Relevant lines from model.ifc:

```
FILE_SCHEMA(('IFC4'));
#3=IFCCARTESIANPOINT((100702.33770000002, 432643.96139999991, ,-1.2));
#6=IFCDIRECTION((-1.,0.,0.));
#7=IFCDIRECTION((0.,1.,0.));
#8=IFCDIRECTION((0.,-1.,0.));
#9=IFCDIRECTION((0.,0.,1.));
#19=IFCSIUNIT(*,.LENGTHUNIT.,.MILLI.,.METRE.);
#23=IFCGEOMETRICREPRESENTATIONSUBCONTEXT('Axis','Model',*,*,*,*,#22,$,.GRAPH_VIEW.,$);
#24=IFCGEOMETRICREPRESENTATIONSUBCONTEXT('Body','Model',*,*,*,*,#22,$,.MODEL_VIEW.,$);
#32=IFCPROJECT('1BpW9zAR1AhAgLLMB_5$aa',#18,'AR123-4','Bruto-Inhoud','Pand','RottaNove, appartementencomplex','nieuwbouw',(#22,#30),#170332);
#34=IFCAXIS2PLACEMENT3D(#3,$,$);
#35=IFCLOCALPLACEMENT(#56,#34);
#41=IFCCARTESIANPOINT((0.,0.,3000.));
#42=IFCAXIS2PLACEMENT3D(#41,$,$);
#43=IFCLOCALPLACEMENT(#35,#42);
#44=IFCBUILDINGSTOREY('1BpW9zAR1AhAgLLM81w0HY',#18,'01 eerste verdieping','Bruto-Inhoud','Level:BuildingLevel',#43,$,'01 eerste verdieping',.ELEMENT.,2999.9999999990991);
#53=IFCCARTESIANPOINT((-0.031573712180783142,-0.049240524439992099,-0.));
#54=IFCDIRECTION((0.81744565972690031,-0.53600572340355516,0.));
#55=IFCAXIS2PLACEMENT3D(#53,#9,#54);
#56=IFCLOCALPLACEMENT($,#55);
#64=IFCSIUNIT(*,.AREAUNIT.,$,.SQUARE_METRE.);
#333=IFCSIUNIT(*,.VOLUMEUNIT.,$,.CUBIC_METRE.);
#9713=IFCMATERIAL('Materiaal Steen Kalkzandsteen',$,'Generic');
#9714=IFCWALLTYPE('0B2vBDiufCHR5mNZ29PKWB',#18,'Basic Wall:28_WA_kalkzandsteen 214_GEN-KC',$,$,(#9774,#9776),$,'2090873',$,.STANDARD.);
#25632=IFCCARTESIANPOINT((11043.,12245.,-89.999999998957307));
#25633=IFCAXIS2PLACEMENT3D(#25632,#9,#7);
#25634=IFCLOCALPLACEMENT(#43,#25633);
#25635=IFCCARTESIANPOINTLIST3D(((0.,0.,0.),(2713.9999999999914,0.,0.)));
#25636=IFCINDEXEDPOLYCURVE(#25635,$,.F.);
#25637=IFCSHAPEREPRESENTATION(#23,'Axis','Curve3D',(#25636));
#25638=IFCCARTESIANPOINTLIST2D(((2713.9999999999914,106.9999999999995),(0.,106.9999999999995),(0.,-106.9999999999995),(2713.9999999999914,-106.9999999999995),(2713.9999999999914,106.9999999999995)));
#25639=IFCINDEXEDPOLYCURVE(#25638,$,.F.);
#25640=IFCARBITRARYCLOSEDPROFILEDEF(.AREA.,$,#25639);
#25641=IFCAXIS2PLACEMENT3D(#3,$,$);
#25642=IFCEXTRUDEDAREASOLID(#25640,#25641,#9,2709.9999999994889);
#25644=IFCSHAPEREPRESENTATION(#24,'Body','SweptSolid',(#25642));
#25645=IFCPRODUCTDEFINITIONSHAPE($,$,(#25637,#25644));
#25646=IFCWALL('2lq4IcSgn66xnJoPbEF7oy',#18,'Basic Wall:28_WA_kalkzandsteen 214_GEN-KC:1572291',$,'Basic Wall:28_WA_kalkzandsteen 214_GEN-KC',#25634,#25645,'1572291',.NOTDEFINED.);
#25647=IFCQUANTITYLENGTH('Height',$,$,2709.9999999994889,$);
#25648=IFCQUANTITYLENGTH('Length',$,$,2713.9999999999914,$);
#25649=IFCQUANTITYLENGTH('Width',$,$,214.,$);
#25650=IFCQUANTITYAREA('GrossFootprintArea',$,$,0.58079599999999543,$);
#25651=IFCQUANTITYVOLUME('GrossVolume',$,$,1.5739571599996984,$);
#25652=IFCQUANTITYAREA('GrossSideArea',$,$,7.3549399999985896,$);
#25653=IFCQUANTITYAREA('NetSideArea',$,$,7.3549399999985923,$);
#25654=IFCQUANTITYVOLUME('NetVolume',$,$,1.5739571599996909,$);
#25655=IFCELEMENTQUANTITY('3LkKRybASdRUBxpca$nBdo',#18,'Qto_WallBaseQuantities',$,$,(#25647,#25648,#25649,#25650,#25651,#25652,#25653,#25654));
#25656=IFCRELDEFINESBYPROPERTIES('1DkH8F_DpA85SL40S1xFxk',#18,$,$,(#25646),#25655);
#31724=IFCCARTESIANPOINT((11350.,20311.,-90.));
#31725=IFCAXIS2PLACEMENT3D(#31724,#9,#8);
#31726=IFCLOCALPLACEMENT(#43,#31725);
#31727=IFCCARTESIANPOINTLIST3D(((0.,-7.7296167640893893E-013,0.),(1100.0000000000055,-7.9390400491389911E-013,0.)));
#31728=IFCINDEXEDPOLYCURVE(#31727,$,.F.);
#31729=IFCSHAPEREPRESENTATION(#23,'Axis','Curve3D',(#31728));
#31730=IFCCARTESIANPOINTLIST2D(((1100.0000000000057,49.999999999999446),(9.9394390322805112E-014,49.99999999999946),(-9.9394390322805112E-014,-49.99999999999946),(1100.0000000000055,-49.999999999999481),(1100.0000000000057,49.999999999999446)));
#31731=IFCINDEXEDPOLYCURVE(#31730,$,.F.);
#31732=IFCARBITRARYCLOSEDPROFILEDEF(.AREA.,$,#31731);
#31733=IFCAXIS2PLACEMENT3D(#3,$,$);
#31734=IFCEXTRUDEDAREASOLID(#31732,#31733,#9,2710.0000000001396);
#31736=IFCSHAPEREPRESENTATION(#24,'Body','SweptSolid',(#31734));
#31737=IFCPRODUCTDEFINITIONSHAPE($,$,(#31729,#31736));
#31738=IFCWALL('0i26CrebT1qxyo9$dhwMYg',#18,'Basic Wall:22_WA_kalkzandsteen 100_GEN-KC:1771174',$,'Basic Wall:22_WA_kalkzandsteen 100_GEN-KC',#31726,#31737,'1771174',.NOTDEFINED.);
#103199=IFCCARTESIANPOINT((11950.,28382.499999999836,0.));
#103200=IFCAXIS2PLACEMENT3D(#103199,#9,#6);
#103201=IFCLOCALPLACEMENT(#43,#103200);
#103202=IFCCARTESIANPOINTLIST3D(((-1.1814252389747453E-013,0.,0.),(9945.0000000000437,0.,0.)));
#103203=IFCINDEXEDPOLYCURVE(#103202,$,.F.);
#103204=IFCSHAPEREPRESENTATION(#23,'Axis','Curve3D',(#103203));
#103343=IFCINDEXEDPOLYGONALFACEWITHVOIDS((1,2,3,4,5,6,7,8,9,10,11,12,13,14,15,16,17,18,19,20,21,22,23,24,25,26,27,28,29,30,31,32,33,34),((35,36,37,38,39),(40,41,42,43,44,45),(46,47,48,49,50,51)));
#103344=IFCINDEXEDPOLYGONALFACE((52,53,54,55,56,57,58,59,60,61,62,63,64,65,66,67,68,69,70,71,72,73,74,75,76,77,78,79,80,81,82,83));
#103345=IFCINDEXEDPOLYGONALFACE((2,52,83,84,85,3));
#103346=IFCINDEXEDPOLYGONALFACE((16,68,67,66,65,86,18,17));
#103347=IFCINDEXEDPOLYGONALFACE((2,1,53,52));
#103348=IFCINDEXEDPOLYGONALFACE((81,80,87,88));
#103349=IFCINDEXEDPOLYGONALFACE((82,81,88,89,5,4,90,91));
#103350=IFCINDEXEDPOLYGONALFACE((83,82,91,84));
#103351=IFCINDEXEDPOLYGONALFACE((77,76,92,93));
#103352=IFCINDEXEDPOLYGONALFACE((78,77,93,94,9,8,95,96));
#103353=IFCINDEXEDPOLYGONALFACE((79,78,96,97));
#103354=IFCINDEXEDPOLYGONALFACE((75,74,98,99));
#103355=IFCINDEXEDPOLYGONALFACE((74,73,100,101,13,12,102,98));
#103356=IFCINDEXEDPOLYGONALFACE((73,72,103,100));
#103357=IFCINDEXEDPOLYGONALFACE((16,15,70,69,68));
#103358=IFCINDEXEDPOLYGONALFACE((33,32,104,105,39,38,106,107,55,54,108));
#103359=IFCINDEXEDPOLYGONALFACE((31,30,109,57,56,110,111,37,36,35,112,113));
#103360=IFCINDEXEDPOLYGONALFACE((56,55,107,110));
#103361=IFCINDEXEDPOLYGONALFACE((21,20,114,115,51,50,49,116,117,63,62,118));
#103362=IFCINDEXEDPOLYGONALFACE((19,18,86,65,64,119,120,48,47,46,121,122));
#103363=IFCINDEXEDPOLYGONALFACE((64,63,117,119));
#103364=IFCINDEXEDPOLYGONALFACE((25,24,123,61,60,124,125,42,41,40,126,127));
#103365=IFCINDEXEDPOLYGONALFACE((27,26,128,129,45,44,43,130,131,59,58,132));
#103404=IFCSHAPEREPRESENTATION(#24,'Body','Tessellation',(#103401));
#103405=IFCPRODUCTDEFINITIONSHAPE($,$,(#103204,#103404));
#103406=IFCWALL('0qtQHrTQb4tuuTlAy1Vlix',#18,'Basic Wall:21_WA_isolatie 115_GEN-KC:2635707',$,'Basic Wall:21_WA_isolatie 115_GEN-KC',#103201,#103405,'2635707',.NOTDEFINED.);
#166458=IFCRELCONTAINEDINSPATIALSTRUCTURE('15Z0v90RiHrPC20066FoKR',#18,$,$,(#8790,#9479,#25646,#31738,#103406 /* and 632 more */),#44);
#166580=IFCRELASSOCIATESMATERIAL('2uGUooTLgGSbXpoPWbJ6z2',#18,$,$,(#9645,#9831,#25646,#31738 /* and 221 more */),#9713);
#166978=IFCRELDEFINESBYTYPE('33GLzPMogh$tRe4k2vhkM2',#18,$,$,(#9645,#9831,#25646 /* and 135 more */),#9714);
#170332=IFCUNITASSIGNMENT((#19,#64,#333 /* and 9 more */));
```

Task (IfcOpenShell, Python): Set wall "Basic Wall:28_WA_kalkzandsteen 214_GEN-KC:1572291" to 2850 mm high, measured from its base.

```python
import ifcopenshell
import ifcopenshell.api.pset
import ifcopenshell.geom
import ifcopenshell.util.element
import ifcopenshell.util.representation
import ifcopenshell.util.shape
import ifcopenshell.util.unit

model = ifcopenshell.open("model.ifc")
unit_scale = ifcopenshell.util.unit.calculate_unit_scale(model)
area_scale = ifcopenshell.util.unit.calculate_unit_scale(model, "AREAUNIT")
volume_scale = ifcopenshell.util.unit.calculate_unit_scale(model, "VOLUMEUNIT")
settings = ifcopenshell.geom.settings()


def volume(element):
    """Net volume in cubic metres, openings subtracted."""
    shape = ifcopenshell.geom.create_shape(settings, element)
    return ifcopenshell.util.shape.get_volume(shape.geometry)


wall = model.by_guid("2lq4IcSgn66xnJoPbEF7oy")
before = volume(wall)

body = ifcopenshell.util.representation.get_representation(wall, "Model", "Body")
solid = body.Items[0]
old_height = solid.Depth
solid.Depth = 2.85 / unit_scale
after = volume(wall)
thickness = 0.214  # wall thickness in metres

# Update the stored height, areas and volumes.
qto = model.by_id(ifcopenshell.util.element.get_pset(wall, "Qto_WallBaseQuantities", should_inherit=False)["id"])
ifcopenshell.api.pset.edit_qto(model, qto=qto, properties={
    "Height": solid.Depth,
    "GrossVolume": ifcopenshell.util.element.get_pset(wall, "Qto_WallBaseQuantities", "GrossVolume") * solid.Depth / old_height,
    "GrossSideArea": ifcopenshell.util.element.get_pset(wall, "Qto_WallBaseQuantities", "GrossSideArea") * solid.Depth / old_height,
    "NetSideArea": after / thickness / area_scale,
    "NetVolume": after / volume_scale,
})

print(f"height {old_height:g} -> {solid.Depth:g}, volume {before:.3f} -> {after:.3f} m3")

model.write("model_rev.ifc")
```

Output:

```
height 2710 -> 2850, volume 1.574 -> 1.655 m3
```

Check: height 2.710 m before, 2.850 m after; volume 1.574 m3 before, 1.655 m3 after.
